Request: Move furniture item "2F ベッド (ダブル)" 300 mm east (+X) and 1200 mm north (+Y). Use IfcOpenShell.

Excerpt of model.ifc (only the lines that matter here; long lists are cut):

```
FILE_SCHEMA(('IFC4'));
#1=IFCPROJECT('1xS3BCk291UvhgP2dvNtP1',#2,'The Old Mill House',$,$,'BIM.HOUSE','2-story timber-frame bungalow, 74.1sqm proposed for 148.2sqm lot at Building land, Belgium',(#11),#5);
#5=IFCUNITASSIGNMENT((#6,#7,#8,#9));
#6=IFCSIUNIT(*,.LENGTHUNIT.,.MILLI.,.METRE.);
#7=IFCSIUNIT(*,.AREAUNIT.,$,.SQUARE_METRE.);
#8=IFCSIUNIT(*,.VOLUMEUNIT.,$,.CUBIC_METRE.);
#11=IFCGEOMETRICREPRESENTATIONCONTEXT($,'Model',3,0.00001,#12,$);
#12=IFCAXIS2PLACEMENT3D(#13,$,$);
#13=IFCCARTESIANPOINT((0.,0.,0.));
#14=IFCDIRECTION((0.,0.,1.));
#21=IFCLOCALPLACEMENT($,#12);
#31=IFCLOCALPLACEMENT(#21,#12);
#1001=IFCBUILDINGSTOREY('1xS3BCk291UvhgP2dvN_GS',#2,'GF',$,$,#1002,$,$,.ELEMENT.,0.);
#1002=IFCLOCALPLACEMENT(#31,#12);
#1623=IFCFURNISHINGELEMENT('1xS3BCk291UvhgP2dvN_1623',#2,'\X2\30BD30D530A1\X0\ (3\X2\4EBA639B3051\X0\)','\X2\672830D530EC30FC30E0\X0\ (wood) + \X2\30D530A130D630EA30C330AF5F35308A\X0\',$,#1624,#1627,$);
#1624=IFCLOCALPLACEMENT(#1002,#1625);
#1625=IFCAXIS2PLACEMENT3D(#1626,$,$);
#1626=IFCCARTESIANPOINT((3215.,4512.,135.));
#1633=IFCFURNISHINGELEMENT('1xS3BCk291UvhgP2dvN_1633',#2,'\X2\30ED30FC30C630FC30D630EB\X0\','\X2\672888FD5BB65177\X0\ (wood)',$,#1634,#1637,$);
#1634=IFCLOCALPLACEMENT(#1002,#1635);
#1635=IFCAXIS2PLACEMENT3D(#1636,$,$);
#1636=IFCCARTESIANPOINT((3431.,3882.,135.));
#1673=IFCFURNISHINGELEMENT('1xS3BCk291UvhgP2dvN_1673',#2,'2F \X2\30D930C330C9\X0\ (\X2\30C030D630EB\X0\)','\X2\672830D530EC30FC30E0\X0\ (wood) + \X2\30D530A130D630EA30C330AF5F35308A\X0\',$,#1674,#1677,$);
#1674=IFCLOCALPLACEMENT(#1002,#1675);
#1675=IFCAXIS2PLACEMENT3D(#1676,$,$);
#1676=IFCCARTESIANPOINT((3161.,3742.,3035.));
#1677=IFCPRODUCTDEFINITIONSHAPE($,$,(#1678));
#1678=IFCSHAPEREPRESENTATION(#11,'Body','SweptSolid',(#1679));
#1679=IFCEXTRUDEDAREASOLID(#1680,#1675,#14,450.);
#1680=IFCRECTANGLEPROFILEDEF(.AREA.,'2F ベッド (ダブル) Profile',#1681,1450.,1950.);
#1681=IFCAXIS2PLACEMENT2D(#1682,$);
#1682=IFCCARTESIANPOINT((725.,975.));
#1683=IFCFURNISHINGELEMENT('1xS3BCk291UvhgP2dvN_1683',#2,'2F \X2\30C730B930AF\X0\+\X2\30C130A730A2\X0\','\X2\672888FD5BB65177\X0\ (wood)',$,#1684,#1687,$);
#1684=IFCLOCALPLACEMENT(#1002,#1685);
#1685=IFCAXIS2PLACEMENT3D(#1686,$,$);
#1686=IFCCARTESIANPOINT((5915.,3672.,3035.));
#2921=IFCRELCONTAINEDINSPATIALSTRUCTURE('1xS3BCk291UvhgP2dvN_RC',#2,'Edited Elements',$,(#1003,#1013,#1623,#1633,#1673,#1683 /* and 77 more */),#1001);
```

```python
import ifcopenshell
import ifcopenshell.api.geometry
import ifcopenshell.util.placement

model = ifcopenshell.open("model.ifc")

item = model.by_id(1673)
matrix = ifcopenshell.util.placement.get_local_placement(item.ObjectPlacement)
matrix[0, 3] += 300.0
matrix[1, 3] += 1200.0
ifcopenshell.api.geometry.edit_object_placement(model, product=item, matrix=matrix, is_si=False)

print(ifcopenshell.util.placement.get_local_placement(item.ObjectPlacement).round(3) + 0.0)

model.write("model_edited.ifc")
```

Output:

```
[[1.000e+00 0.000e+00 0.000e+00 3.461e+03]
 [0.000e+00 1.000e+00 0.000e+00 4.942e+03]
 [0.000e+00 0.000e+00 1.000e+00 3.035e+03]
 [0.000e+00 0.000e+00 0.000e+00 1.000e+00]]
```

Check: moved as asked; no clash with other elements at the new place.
